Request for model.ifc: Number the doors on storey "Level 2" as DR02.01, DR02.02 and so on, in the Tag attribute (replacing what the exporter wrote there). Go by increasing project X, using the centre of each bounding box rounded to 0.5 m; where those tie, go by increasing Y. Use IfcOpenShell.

First a look at what the model holds.

```python
import ifcopenshell
import ifcopenshell.util.element
import ifcopenshell.util.placement

model = ifcopenshell.open("model.ifc")
print(model.schema)
storey = next(s for s in model.by_type("IfcBuildingStorey") if s.Name == "Level 2")
doors = [e for e in ifcopenshell.util.element.get_decomposition(storey) if e.is_a("IfcDoor")]
for e in sorted(doors, key=lambda e: e.id()):
    origin = ifcopenshell.util.placement.get_local_placement(e.ObjectPlacement)[:3, 3]
    print(e.id(), e.Tag, e.Name, origin.round(2) + 0.0, sep=" | ")
```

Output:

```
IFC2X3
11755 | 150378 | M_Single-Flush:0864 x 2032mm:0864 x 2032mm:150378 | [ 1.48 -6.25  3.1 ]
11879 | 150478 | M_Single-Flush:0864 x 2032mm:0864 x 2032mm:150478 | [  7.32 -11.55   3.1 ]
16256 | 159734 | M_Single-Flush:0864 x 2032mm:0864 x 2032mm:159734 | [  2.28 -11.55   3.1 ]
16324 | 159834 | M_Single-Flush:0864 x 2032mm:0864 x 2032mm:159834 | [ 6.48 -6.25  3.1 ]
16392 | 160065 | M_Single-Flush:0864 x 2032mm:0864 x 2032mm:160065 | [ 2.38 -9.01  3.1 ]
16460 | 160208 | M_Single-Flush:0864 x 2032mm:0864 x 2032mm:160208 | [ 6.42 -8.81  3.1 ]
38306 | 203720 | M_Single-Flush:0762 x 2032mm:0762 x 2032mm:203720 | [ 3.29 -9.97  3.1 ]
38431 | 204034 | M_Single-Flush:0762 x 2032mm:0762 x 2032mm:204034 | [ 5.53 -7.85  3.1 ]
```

```python
import ifcopenshell
import ifcopenshell.geom
import ifcopenshell.util.element
import ifcopenshell.util.shape

model = ifcopenshell.open("model.ifc")
settings = ifcopenshell.geom.settings()
settings.set("use-world-coords", True)


def centre(element):
    shape = ifcopenshell.geom.create_shape(settings, element)
    return ifcopenshell.util.shape.get_bbox_centroid(shape.geometry)


storey = next(s for s in model.by_type("IfcBuildingStorey") if s.Name == "Level 2")
doors = [e for e in ifcopenshell.util.element.get_decomposition(storey) if e.is_a("IfcDoor")]

# Insertion points can sit at a corner or the storey origin, so sort by the geometry (in metres).
centres = {e: centre(e) for e in doors}
doors.sort(key=lambda e: (round(centres[e][0] / 0.5), centres[e][1]))

for i, e in enumerate(doors, start=1):
    number = f"DR02.{i:02d}"
    e.Tag = number
    print(e.id(), number)

model.write("model_edited.ifc")
```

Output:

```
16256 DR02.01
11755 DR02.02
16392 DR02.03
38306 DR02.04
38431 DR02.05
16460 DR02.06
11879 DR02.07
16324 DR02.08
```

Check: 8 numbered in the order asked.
